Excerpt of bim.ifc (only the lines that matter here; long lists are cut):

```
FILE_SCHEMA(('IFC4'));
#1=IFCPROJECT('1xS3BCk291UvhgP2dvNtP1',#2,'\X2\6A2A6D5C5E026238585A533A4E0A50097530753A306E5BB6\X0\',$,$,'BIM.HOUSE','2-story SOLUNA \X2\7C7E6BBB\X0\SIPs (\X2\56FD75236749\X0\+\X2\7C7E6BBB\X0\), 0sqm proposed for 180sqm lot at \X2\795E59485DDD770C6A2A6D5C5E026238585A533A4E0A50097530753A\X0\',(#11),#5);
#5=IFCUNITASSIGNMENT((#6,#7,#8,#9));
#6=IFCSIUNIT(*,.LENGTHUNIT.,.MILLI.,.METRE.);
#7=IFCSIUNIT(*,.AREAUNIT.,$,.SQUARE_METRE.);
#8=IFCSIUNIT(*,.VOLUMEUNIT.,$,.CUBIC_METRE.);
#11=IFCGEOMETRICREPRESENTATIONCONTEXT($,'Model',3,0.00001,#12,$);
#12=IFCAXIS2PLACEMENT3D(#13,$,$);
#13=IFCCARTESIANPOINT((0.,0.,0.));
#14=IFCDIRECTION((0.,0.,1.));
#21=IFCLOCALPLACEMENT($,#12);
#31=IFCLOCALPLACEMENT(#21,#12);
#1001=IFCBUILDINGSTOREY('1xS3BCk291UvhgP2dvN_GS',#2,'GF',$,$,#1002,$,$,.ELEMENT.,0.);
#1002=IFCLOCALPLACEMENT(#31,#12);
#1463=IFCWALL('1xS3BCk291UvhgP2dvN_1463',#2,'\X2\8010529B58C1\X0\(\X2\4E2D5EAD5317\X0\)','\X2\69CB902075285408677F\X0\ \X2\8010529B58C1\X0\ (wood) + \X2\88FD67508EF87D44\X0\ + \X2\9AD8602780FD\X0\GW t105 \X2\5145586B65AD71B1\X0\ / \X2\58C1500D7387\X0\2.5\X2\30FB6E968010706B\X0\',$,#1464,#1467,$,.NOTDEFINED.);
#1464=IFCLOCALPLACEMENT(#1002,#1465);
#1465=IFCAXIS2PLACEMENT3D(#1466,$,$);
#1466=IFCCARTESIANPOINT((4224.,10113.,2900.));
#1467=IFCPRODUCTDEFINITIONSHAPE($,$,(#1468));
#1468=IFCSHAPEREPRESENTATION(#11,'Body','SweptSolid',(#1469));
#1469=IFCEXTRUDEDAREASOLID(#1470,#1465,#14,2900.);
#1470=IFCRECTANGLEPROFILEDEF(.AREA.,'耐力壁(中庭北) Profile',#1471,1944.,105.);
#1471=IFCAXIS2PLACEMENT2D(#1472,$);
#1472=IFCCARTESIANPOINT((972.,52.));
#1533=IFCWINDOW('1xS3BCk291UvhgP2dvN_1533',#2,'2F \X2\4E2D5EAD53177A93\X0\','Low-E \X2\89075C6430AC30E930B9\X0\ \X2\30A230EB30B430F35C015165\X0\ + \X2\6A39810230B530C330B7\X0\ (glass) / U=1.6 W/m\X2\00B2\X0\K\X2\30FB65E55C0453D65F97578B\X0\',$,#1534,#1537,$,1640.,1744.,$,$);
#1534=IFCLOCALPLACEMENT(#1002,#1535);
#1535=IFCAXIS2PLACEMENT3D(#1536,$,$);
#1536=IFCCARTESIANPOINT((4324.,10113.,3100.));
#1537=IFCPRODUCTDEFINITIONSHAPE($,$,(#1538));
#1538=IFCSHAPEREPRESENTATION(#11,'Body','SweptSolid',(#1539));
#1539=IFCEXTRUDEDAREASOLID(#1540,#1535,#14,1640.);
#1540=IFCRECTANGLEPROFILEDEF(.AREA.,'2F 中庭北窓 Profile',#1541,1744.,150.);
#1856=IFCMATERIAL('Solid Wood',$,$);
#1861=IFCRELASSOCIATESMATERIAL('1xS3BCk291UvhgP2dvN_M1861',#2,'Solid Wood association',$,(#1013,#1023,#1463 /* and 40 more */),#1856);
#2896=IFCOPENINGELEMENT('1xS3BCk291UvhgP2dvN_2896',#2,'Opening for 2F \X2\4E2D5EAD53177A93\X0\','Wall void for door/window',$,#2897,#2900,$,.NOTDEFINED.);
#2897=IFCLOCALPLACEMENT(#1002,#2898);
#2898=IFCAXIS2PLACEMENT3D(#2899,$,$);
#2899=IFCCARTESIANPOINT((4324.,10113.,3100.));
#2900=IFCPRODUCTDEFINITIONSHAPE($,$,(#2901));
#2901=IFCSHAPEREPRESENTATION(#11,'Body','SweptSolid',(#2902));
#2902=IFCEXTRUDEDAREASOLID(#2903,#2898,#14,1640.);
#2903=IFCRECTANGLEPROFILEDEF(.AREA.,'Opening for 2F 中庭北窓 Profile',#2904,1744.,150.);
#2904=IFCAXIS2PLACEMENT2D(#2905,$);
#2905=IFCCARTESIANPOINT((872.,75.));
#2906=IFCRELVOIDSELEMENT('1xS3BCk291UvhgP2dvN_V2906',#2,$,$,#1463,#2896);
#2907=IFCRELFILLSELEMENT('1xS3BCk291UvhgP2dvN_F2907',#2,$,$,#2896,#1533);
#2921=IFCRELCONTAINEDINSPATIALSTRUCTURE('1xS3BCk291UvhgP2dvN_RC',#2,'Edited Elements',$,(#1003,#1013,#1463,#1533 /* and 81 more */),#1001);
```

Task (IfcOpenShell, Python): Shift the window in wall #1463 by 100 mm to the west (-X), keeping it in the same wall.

```python
import ifcopenshell
import ifcopenshell.api.geometry
import ifcopenshell.util.placement

model = ifcopenshell.open("bim.ifc")

window = model.by_id(1533)
opening = window.FillsVoids[0].RelatingOpeningElement
wall = opening.VoidsElements[0].RelatingBuildingElement

wall_matrix = ifcopenshell.util.placement.get_local_placement(wall.ObjectPlacement)
shift = wall_matrix[:3, 0] * -100.0
before = ifcopenshell.util.placement.get_local_placement(window.ObjectPlacement)[:3, 3].copy()

# The window is not placed relative to its opening, so move both.
for product in (opening, window):
    matrix = ifcopenshell.util.placement.get_local_placement(product.ObjectPlacement)
    matrix[:3, 3] += shift
    ifcopenshell.api.geometry.edit_object_placement(model, product=product, matrix=matrix, is_si=False)

after = ifcopenshell.util.placement.get_local_placement(window.ObjectPlacement)[:3, 3]
print("window moved by", (after - before).round(3) + 0.0)

model.write("bim_edited.ifc")
```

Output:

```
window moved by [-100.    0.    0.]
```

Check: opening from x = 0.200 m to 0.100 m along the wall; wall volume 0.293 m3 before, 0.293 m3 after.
